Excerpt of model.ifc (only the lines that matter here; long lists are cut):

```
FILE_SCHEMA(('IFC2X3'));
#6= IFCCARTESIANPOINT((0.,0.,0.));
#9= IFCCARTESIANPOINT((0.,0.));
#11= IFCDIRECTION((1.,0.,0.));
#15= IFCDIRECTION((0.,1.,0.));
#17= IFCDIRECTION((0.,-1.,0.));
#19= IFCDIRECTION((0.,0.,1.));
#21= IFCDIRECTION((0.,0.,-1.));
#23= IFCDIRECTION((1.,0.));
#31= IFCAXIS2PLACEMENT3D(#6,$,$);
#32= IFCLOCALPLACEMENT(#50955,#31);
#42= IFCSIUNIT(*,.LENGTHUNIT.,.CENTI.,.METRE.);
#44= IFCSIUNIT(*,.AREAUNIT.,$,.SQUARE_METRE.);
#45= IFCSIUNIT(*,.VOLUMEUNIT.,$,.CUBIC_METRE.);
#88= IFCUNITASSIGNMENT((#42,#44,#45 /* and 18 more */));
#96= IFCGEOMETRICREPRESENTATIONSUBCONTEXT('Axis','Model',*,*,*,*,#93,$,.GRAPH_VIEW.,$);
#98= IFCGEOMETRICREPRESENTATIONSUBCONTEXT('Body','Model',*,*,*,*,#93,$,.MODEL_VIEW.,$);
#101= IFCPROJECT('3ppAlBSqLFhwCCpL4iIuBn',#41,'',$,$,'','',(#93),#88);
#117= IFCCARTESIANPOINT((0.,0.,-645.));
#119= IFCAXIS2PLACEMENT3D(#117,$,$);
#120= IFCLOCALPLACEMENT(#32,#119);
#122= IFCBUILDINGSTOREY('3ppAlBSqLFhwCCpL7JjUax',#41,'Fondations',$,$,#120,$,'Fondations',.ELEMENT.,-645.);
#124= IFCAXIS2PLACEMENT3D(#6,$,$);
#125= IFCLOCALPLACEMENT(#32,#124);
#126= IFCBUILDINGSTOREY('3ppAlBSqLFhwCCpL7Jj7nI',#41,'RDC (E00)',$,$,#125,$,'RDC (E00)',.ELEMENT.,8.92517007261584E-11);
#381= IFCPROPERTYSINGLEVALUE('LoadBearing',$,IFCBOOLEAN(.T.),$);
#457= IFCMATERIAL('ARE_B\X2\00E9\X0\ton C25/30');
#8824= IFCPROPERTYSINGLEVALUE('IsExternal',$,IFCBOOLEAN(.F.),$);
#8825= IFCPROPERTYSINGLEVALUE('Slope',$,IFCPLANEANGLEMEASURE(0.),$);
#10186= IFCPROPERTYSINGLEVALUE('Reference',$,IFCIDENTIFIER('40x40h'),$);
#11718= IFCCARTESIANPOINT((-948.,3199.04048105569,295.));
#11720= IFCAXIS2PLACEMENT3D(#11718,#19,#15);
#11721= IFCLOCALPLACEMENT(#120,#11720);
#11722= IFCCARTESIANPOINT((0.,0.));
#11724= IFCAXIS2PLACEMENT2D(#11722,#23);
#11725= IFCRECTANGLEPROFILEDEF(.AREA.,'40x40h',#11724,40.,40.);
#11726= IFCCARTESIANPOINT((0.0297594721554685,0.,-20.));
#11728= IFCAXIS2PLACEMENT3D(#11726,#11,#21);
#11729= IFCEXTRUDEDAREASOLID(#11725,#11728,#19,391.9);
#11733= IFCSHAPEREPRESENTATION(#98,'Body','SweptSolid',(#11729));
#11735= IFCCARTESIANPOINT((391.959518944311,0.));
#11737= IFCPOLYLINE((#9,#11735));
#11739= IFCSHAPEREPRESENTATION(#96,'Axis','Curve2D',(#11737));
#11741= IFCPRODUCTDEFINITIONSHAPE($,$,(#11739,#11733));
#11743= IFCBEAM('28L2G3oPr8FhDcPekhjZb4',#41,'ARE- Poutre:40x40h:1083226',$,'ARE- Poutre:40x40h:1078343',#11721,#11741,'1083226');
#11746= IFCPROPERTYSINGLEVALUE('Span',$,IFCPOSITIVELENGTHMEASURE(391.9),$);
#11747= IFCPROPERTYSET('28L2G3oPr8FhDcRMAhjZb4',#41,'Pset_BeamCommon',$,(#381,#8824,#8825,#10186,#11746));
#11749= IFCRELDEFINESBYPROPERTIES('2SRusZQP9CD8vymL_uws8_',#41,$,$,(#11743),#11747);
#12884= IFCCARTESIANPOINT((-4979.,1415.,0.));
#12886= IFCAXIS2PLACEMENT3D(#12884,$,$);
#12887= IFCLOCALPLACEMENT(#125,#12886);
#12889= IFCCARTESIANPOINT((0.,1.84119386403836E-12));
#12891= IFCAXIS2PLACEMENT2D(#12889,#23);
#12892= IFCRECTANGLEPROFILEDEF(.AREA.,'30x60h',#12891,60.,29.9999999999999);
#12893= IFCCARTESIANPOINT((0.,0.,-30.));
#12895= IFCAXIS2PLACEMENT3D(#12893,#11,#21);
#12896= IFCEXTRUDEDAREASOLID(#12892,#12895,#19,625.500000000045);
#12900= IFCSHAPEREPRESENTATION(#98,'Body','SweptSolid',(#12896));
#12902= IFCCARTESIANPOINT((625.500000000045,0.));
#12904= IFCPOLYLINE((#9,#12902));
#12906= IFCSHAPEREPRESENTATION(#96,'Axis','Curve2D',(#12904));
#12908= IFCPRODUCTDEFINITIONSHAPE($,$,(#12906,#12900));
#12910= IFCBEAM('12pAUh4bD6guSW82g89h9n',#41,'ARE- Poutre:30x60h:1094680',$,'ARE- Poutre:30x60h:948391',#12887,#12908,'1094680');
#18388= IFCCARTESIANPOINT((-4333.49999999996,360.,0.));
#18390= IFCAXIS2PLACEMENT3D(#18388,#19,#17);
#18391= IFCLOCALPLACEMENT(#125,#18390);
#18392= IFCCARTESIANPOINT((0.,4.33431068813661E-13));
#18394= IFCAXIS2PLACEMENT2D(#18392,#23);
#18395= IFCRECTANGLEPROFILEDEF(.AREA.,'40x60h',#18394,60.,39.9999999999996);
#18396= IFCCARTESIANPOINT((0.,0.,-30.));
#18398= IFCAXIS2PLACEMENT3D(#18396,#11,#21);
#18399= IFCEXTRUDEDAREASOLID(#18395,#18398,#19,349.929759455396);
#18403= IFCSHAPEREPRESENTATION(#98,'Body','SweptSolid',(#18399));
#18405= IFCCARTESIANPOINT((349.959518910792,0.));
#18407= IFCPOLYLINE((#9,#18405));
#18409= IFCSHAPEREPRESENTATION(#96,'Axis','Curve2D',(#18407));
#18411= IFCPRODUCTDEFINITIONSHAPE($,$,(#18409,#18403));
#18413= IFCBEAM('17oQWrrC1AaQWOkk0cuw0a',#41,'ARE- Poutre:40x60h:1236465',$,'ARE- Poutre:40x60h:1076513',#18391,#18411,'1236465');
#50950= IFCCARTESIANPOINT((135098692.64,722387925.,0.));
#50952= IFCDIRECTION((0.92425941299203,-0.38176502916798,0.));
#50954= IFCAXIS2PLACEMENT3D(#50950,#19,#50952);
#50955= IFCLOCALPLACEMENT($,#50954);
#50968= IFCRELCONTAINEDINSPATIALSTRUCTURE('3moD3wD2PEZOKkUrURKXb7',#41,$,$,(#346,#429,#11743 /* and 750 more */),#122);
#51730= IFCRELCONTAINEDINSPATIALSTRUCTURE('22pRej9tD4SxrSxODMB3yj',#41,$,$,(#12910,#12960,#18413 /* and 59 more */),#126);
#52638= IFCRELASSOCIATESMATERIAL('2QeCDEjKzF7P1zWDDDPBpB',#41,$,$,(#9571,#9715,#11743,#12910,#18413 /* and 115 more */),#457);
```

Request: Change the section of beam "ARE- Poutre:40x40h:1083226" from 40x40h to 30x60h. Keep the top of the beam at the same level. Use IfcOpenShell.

```python
import ifcopenshell
import ifcopenshell.api.pset
import ifcopenshell.util.element
import ifcopenshell.util.representation

model = ifcopenshell.open("model.ifc")

member = model.by_guid("28L2G3oPr8FhDcPekhjZb4")
source = next(p for p in model.by_type("IfcRectangleProfileDef") if p.ProfileName == "30x60h")

body = ifcopenshell.util.representation.get_representation(member, "Model", "Body")
solid = body.Items[0]
old_profile = solid.SweptArea

# Copy the section's sizes but keep this member's own profile position.
profile = ifcopenshell.util.element.copy(model, source)
# Profiles are centred, so shift by half the change in depth to hold the top.
shift = (old_profile.XDim - profile.XDim) / 2
x, y = old_profile.Position.Location.Coordinates
up = (-1.0, 0.0)  # upwards, in the solid's own plane
location = model.createIfcCartesianPoint((x + up[0] * shift, y + up[1] * shift))
profile.Position = model.createIfcAxis2Placement2D(location, old_profile.Position.RefDirection)
solid.SweptArea = profile
if not model.get_total_inverses(old_profile):
    ifcopenshell.util.element.remove_deep2(model, old_profile)
member.Name = member.Name.replace("40x40h", "30x60h")
member.ObjectType = member.ObjectType.replace("40x40h", "30x60h")
pset = model.by_id(ifcopenshell.util.element.get_pset(member, "Pset_BeamCommon", should_inherit=False)["id"])
ifcopenshell.api.pset.edit_pset(model, pset=pset, properties={"Reference": "30x60h"})

print(solid.SweptArea)

model.write("model_v2.ifc")
```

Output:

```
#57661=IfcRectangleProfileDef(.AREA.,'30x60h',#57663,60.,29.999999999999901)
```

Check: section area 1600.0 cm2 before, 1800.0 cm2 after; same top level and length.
